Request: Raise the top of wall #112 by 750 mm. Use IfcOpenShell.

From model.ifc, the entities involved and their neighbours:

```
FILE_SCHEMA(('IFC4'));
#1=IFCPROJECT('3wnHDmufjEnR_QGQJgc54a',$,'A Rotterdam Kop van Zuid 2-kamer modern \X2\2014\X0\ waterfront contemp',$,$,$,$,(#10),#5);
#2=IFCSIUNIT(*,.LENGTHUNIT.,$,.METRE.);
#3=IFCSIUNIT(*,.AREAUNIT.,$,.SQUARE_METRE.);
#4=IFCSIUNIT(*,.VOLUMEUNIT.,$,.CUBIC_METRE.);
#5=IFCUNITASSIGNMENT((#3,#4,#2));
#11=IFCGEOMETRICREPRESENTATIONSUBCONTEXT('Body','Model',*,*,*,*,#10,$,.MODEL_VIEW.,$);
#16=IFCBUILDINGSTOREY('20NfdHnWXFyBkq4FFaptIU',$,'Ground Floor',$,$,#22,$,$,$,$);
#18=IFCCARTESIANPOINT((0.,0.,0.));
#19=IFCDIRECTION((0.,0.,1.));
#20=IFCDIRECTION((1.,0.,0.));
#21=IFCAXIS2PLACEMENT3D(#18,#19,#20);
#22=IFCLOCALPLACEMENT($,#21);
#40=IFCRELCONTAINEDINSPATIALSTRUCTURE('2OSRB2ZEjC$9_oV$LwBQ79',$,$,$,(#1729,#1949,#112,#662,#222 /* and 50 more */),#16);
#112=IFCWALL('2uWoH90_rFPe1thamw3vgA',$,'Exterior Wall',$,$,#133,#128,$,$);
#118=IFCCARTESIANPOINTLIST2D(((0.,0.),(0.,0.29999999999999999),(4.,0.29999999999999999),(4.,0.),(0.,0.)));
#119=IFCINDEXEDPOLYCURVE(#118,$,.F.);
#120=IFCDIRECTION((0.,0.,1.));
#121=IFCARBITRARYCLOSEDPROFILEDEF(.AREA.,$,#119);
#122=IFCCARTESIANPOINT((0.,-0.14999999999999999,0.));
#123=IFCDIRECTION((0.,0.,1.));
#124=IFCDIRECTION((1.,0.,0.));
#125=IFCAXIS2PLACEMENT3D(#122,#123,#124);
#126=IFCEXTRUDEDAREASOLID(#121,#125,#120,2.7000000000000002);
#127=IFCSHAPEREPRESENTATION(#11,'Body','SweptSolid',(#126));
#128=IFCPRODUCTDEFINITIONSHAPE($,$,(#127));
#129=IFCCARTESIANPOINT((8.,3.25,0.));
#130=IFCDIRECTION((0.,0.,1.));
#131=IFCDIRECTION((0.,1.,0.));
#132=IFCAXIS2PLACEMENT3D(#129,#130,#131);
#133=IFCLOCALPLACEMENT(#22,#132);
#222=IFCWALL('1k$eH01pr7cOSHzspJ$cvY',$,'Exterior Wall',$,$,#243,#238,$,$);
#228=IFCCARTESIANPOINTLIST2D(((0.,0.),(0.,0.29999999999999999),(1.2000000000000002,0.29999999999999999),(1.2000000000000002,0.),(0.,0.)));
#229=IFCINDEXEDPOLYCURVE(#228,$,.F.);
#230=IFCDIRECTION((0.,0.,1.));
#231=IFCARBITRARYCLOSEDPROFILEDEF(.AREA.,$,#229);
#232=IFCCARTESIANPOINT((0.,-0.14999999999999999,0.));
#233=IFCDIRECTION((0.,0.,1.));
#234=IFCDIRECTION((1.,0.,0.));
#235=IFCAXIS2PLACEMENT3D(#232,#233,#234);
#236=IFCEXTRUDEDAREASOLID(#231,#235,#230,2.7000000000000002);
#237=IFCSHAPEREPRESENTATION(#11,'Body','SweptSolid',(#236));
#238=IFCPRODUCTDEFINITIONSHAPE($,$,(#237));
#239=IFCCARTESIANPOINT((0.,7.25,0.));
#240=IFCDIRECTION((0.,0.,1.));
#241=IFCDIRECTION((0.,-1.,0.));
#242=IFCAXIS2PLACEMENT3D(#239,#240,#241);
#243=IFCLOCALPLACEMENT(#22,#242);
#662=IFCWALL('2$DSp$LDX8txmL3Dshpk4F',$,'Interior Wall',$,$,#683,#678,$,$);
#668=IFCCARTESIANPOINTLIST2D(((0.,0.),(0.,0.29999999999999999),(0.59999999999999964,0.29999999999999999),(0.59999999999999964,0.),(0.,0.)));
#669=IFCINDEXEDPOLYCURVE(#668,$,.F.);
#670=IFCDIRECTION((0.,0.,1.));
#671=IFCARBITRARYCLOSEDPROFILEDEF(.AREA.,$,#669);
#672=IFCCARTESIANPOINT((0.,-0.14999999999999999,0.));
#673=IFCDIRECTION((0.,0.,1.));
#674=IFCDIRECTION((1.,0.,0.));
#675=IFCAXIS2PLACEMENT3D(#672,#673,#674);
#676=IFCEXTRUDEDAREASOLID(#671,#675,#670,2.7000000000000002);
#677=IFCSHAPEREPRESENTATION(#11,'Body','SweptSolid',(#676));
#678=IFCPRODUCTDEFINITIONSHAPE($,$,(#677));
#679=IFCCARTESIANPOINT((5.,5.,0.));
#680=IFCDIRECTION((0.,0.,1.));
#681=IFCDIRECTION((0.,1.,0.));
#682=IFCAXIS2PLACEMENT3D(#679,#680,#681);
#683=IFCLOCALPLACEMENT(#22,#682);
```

```python
import ifcopenshell
import ifcopenshell.geom
import ifcopenshell.util.representation
import ifcopenshell.util.shape

model = ifcopenshell.open("model.ifc")
settings = ifcopenshell.geom.settings()


def volume(element):
    """Net volume in cubic metres, openings subtracted."""
    shape = ifcopenshell.geom.create_shape(settings, element)
    return ifcopenshell.util.shape.get_volume(shape.geometry)


wall = model.by_id(112)
before = volume(wall)

body = ifcopenshell.util.representation.get_representation(wall, "Model", "Body")
solid = body.Items[0]
old_height = solid.Depth
solid.Depth += 0.75
after = volume(wall)

print(f"height {old_height:g} -> {solid.Depth:g}, volume {before:.3f} -> {after:.3f} m3")

model.write("model_v2.ifc")
```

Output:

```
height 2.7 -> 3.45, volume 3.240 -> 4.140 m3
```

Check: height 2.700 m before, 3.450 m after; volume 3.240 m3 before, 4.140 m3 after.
